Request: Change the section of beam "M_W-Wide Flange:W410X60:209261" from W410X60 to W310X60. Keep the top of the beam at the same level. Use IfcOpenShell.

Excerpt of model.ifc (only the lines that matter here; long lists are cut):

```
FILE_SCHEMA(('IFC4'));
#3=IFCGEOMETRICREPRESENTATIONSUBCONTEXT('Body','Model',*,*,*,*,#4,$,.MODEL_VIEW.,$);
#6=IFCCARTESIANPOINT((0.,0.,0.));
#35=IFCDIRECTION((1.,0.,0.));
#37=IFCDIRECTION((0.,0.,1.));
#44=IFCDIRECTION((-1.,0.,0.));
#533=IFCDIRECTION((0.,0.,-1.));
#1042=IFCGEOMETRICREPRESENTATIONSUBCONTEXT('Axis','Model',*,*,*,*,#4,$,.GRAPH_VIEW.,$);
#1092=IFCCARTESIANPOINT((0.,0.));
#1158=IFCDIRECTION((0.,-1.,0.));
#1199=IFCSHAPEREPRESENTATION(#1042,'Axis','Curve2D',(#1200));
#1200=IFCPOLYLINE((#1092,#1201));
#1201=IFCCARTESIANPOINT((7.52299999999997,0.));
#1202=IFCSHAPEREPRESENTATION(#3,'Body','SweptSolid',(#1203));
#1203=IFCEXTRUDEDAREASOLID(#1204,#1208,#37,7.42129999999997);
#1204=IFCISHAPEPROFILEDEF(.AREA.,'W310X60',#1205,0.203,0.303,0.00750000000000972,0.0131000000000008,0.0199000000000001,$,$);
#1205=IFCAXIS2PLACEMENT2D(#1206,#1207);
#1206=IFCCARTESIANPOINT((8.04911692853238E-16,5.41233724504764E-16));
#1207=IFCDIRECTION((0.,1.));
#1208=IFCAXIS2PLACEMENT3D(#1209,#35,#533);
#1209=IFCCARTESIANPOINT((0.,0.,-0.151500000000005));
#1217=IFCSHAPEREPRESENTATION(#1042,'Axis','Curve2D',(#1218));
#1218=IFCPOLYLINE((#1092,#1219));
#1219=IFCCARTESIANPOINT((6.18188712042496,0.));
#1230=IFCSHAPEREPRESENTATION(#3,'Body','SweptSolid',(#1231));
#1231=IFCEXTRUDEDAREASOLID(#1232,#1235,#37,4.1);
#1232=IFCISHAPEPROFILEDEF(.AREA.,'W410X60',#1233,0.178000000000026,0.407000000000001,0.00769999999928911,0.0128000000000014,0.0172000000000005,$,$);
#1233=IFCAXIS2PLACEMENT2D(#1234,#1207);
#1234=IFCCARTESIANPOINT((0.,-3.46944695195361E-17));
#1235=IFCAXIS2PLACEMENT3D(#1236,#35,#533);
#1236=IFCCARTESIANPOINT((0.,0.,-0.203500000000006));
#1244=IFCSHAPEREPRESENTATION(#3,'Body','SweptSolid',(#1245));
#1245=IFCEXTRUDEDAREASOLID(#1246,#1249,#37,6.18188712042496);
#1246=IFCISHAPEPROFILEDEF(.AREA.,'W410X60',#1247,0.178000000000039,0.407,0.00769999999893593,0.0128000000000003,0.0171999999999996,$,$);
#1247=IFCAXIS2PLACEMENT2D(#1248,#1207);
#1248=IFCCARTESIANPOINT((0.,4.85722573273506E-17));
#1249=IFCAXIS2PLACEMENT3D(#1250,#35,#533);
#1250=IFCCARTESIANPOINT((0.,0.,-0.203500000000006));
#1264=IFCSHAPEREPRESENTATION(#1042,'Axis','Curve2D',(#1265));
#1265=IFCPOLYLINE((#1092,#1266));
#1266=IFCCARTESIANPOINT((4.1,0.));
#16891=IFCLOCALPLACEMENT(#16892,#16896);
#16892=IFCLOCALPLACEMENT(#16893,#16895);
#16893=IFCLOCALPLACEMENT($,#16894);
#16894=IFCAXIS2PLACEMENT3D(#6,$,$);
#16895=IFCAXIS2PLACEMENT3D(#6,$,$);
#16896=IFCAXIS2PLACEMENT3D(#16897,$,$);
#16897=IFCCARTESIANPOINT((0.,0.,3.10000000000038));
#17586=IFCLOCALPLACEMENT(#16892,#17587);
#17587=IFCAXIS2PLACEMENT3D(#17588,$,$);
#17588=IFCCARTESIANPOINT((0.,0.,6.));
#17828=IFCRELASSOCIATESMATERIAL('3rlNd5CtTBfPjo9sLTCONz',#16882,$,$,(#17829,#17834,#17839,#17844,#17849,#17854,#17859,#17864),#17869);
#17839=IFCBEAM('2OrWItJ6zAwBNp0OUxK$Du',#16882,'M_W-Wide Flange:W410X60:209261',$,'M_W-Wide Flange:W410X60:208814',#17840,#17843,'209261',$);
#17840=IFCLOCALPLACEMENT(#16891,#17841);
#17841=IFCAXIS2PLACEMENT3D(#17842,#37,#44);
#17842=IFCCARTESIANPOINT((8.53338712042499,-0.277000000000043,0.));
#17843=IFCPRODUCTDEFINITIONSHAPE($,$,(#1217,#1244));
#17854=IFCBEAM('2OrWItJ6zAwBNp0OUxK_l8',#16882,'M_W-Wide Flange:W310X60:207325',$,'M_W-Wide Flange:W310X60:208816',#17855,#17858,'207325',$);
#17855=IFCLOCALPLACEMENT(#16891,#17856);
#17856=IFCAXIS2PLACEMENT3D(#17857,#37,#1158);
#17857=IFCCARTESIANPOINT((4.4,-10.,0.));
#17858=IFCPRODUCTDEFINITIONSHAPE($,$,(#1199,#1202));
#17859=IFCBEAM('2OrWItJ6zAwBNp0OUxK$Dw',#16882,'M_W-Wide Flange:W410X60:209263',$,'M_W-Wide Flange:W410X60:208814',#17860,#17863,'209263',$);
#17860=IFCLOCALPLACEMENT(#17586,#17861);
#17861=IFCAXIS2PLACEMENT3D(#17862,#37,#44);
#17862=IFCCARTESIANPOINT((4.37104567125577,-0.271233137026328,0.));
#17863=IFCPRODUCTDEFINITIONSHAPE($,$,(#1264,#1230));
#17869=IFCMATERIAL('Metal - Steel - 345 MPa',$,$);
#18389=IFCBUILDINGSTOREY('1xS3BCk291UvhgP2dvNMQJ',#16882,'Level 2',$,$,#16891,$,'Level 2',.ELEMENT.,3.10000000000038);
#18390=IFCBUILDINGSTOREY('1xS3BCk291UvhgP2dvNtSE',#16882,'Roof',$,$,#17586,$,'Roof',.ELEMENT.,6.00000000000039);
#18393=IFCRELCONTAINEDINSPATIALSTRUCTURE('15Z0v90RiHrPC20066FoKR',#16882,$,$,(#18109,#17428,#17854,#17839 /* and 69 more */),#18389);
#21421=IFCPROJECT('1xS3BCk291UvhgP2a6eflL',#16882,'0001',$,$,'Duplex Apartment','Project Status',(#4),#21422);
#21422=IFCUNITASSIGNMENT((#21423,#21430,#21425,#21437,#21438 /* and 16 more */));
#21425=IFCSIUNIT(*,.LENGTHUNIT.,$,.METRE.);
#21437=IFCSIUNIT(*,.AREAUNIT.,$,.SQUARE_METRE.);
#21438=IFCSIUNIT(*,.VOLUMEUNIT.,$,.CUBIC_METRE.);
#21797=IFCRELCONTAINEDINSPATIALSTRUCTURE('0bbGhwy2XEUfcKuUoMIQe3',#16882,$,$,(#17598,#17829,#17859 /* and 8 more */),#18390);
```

```python
import ifcopenshell
import ifcopenshell.util.element
import ifcopenshell.util.representation

model = ifcopenshell.open("model.ifc")

member = model.by_guid("2OrWItJ6zAwBNp0OUxK$Du")
source = next(p for p in model.by_type("IfcIShapeProfileDef") if p.ProfileName == "W310X60")

body = ifcopenshell.util.representation.get_representation(member, "Model", "Body")
solid = body.Items[0]
old_profile = solid.SweptArea

# Copy the section's sizes but keep this member's own profile position.
profile = ifcopenshell.util.element.copy(model, source)
# Profiles are centred, so shift by half the change in depth to hold the top.
shift = (old_profile.OverallDepth - profile.OverallDepth) / 2
x, y = old_profile.Position.Location.Coordinates
up = (-1.0, 0.0)  # upwards, in the solid's own plane
location = model.createIfcCartesianPoint((x + up[0] * shift, y + up[1] * shift))
profile.Position = model.createIfcAxis2Placement2D(location, old_profile.Position.RefDirection)
solid.SweptArea = profile
if not model.get_total_inverses(old_profile):
    ifcopenshell.util.element.remove_deep2(model, old_profile)
member.Name = member.Name.replace("W410X60", "W310X60")
member.ObjectType = member.ObjectType.replace("W410X60", "W310X60")

print(solid.SweptArea)

model.write("model_rev.ifc")
```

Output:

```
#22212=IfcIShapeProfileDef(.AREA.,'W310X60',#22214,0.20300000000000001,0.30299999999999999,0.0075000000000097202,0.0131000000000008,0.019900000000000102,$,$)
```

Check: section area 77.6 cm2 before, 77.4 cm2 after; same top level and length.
